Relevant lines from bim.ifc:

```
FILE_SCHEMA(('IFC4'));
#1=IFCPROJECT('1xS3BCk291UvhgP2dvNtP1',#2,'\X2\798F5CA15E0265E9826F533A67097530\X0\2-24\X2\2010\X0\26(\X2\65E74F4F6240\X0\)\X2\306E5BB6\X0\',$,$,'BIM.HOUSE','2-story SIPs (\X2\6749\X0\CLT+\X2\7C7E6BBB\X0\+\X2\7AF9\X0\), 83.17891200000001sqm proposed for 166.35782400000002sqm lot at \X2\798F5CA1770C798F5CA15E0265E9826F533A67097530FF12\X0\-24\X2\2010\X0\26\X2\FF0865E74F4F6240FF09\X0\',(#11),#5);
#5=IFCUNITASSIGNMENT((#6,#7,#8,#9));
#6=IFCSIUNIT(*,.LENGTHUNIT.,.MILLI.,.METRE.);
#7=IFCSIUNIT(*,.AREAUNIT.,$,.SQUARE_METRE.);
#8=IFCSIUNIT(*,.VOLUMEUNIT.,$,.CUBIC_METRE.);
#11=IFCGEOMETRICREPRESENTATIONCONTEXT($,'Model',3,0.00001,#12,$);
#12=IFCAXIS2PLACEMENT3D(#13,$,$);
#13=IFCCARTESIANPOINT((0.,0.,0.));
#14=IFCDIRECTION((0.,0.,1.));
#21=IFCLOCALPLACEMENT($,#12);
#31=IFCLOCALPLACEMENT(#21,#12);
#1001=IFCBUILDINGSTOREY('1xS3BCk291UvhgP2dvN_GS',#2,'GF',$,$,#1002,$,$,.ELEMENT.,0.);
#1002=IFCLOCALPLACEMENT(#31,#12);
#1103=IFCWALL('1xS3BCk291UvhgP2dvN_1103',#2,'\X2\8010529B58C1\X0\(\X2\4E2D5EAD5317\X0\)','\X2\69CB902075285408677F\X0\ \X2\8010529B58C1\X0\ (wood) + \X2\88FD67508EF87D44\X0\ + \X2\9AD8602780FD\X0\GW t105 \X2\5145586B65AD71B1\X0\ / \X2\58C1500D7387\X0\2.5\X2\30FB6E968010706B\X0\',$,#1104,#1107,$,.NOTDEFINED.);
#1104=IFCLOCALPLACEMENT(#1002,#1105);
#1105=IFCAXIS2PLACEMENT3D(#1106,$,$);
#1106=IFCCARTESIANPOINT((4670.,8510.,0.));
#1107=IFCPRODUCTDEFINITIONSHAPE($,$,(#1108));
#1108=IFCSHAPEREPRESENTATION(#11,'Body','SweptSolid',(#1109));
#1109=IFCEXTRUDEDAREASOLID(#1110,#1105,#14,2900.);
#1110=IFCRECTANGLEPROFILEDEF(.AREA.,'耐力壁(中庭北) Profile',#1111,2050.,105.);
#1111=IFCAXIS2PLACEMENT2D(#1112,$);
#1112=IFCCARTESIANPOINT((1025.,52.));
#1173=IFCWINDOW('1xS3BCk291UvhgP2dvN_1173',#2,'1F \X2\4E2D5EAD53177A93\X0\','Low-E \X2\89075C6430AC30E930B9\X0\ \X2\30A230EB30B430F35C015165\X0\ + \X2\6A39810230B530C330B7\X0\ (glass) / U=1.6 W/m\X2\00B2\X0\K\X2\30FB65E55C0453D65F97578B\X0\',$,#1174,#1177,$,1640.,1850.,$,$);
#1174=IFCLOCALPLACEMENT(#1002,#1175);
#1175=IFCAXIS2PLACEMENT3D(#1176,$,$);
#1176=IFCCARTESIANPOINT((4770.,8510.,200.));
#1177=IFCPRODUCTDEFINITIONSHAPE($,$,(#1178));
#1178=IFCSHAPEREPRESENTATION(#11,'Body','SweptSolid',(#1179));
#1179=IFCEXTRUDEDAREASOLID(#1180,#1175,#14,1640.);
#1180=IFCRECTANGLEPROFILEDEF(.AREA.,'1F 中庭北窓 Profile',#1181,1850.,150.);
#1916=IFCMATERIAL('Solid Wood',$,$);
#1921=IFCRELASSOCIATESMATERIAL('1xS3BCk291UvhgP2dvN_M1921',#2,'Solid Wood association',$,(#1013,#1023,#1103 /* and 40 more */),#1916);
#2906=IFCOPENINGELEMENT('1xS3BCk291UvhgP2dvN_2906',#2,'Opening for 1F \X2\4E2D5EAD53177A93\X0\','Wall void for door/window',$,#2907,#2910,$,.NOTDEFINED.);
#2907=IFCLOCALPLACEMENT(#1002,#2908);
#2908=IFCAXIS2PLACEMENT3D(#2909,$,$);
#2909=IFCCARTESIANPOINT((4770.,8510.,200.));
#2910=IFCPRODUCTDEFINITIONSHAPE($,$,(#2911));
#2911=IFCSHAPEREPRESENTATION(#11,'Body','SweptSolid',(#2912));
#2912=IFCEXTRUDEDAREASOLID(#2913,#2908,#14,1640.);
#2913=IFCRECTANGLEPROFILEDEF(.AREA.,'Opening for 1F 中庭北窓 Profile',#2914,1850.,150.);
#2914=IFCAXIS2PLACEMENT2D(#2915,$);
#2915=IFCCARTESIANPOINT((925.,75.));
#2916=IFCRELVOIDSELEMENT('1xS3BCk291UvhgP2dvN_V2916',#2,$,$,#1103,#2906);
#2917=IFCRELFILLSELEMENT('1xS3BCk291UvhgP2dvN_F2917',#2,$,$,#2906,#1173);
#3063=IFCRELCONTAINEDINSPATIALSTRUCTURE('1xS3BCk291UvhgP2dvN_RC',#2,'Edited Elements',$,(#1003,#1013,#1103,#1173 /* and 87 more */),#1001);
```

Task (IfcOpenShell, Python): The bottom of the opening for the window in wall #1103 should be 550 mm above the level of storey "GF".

```python
import numpy as np
import ifcopenshell
import ifcopenshell.api.geometry
import ifcopenshell.geom
import ifcopenshell.util.element
import ifcopenshell.util.placement
import ifcopenshell.util.shape
import ifcopenshell.util.unit

model = ifcopenshell.open("bim.ifc")
unit_scale = ifcopenshell.util.unit.calculate_unit_scale(model)

window = model.by_id(1173)
opening = window.FillsVoids[0].RelatingOpeningElement
storey = ifcopenshell.util.element.get_container(window, ifc_class="IfcBuildingStorey")
level = ifcopenshell.util.placement.get_local_placement(storey.ObjectPlacement)[2, 3]

# The opening's origin need not be at the sill, so measure its lowest point.
shape = ifcopenshell.geom.create_shape(ifcopenshell.geom.settings(), opening)
bottom = ifcopenshell.util.shape.get_shape_bottom_elevation(shape, shape.geometry) / unit_scale
dz = level + 0.55 / unit_scale - bottom

shift = np.array([0.0, 0.0, dz])
# The window is not placed relative to its opening, so move both.
for product in (opening, window):
    matrix = ifcopenshell.util.placement.get_local_placement(product.ObjectPlacement)
    matrix[:3, 3] += shift
    ifcopenshell.api.geometry.edit_object_placement(model, product=product, matrix=matrix, is_si=False)

print(f"moved by {dz * unit_scale:+.3f} m")

model.write("bim_rev.ifc")
```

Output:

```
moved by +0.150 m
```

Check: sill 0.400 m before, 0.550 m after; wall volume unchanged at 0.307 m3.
